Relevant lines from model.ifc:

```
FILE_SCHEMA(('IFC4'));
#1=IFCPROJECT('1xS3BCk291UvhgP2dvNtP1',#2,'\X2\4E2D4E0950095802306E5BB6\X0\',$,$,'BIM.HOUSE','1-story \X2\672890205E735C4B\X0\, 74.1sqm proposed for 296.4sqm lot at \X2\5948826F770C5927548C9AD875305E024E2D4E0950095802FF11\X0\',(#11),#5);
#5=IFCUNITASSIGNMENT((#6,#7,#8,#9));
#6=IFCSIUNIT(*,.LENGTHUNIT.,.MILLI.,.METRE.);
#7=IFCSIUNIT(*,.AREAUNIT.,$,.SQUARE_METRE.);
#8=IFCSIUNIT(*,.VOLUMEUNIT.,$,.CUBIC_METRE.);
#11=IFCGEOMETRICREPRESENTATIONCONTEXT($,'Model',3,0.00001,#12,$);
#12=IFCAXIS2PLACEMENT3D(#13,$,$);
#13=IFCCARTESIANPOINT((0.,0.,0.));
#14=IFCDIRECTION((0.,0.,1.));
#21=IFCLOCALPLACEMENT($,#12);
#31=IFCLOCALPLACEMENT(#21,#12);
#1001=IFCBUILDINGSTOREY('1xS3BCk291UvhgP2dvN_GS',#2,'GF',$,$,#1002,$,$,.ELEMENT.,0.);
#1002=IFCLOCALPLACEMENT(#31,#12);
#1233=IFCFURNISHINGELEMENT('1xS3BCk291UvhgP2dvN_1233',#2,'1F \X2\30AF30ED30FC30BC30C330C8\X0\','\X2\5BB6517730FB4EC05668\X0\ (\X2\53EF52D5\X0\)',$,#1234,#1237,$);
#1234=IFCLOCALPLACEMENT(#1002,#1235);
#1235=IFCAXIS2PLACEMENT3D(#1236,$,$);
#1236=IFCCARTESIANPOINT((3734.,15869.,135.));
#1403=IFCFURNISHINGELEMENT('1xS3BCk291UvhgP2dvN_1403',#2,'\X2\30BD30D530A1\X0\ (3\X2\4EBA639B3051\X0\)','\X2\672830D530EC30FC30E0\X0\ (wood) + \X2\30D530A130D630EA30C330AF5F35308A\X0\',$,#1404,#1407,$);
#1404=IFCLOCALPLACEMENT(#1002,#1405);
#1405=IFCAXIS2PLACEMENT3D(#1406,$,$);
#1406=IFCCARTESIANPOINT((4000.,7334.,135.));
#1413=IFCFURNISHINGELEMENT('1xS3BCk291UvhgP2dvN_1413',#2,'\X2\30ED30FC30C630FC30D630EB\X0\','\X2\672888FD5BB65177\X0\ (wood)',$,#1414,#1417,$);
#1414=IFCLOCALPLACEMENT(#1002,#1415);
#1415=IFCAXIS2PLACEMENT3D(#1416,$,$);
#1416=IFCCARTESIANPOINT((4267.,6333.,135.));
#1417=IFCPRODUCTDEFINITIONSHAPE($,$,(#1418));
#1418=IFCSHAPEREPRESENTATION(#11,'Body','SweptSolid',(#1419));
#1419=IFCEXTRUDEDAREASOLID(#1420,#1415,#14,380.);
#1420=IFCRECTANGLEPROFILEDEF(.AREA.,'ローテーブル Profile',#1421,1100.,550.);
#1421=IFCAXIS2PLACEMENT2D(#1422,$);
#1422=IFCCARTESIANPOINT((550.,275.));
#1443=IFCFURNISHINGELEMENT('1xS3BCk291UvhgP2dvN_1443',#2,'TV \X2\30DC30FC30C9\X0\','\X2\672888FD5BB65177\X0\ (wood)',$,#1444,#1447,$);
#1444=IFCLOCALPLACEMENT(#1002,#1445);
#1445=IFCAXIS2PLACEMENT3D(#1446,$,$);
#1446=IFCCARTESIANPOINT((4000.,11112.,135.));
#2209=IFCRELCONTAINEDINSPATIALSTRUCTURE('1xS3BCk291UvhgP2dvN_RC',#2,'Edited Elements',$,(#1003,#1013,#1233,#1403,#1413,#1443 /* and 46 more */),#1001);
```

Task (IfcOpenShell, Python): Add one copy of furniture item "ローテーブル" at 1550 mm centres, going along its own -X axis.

```python
import ifcopenshell
import ifcopenshell.api.geometry
import ifcopenshell.api.root
import ifcopenshell.util.element
import ifcopenshell.util.placement
import ifcopenshell.util.unit

model = ifcopenshell.open("model.ifc")
unit_scale = ifcopenshell.util.unit.calculate_unit_scale(model)


def reuse_history(source, copy):
    """copy_class also copies each property set's owner history, people and application; keep the originals."""
    for rel in copy.IsDefinedBy:
        if rel.is_a("IfcRelDefinesByProperties") and (history := rel.RelatingPropertyDefinition.OwnerHistory):
            rel.RelatingPropertyDefinition.OwnerHistory = source.OwnerHistory
            ifcopenshell.util.element.remove_deep2(model, history)


source = model.by_id(1413)
base = ifcopenshell.util.placement.get_local_placement(source.ObjectPlacement)
step = -base[:3, 0] * 1.55 / unit_scale

for i in range(1, 2):
    copy = ifcopenshell.api.root.copy_class(model, product=source)
    copy.Representation = ifcopenshell.util.element.copy_deep(
        model, source.Representation, exclude=["IfcGeometricRepresentationContext", "IfcRepresentationMap"]
    )
    reuse_history(source, copy)
    matrix = base.copy()
    matrix[:3, 3] += i * step
    print("added at", matrix[:3, 3].round(3) + 0.0)
    ifcopenshell.api.geometry.edit_object_placement(model, product=copy, matrix=matrix, is_si=False)

model.write("model_edited.ifc")
```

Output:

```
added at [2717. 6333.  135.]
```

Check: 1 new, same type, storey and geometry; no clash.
